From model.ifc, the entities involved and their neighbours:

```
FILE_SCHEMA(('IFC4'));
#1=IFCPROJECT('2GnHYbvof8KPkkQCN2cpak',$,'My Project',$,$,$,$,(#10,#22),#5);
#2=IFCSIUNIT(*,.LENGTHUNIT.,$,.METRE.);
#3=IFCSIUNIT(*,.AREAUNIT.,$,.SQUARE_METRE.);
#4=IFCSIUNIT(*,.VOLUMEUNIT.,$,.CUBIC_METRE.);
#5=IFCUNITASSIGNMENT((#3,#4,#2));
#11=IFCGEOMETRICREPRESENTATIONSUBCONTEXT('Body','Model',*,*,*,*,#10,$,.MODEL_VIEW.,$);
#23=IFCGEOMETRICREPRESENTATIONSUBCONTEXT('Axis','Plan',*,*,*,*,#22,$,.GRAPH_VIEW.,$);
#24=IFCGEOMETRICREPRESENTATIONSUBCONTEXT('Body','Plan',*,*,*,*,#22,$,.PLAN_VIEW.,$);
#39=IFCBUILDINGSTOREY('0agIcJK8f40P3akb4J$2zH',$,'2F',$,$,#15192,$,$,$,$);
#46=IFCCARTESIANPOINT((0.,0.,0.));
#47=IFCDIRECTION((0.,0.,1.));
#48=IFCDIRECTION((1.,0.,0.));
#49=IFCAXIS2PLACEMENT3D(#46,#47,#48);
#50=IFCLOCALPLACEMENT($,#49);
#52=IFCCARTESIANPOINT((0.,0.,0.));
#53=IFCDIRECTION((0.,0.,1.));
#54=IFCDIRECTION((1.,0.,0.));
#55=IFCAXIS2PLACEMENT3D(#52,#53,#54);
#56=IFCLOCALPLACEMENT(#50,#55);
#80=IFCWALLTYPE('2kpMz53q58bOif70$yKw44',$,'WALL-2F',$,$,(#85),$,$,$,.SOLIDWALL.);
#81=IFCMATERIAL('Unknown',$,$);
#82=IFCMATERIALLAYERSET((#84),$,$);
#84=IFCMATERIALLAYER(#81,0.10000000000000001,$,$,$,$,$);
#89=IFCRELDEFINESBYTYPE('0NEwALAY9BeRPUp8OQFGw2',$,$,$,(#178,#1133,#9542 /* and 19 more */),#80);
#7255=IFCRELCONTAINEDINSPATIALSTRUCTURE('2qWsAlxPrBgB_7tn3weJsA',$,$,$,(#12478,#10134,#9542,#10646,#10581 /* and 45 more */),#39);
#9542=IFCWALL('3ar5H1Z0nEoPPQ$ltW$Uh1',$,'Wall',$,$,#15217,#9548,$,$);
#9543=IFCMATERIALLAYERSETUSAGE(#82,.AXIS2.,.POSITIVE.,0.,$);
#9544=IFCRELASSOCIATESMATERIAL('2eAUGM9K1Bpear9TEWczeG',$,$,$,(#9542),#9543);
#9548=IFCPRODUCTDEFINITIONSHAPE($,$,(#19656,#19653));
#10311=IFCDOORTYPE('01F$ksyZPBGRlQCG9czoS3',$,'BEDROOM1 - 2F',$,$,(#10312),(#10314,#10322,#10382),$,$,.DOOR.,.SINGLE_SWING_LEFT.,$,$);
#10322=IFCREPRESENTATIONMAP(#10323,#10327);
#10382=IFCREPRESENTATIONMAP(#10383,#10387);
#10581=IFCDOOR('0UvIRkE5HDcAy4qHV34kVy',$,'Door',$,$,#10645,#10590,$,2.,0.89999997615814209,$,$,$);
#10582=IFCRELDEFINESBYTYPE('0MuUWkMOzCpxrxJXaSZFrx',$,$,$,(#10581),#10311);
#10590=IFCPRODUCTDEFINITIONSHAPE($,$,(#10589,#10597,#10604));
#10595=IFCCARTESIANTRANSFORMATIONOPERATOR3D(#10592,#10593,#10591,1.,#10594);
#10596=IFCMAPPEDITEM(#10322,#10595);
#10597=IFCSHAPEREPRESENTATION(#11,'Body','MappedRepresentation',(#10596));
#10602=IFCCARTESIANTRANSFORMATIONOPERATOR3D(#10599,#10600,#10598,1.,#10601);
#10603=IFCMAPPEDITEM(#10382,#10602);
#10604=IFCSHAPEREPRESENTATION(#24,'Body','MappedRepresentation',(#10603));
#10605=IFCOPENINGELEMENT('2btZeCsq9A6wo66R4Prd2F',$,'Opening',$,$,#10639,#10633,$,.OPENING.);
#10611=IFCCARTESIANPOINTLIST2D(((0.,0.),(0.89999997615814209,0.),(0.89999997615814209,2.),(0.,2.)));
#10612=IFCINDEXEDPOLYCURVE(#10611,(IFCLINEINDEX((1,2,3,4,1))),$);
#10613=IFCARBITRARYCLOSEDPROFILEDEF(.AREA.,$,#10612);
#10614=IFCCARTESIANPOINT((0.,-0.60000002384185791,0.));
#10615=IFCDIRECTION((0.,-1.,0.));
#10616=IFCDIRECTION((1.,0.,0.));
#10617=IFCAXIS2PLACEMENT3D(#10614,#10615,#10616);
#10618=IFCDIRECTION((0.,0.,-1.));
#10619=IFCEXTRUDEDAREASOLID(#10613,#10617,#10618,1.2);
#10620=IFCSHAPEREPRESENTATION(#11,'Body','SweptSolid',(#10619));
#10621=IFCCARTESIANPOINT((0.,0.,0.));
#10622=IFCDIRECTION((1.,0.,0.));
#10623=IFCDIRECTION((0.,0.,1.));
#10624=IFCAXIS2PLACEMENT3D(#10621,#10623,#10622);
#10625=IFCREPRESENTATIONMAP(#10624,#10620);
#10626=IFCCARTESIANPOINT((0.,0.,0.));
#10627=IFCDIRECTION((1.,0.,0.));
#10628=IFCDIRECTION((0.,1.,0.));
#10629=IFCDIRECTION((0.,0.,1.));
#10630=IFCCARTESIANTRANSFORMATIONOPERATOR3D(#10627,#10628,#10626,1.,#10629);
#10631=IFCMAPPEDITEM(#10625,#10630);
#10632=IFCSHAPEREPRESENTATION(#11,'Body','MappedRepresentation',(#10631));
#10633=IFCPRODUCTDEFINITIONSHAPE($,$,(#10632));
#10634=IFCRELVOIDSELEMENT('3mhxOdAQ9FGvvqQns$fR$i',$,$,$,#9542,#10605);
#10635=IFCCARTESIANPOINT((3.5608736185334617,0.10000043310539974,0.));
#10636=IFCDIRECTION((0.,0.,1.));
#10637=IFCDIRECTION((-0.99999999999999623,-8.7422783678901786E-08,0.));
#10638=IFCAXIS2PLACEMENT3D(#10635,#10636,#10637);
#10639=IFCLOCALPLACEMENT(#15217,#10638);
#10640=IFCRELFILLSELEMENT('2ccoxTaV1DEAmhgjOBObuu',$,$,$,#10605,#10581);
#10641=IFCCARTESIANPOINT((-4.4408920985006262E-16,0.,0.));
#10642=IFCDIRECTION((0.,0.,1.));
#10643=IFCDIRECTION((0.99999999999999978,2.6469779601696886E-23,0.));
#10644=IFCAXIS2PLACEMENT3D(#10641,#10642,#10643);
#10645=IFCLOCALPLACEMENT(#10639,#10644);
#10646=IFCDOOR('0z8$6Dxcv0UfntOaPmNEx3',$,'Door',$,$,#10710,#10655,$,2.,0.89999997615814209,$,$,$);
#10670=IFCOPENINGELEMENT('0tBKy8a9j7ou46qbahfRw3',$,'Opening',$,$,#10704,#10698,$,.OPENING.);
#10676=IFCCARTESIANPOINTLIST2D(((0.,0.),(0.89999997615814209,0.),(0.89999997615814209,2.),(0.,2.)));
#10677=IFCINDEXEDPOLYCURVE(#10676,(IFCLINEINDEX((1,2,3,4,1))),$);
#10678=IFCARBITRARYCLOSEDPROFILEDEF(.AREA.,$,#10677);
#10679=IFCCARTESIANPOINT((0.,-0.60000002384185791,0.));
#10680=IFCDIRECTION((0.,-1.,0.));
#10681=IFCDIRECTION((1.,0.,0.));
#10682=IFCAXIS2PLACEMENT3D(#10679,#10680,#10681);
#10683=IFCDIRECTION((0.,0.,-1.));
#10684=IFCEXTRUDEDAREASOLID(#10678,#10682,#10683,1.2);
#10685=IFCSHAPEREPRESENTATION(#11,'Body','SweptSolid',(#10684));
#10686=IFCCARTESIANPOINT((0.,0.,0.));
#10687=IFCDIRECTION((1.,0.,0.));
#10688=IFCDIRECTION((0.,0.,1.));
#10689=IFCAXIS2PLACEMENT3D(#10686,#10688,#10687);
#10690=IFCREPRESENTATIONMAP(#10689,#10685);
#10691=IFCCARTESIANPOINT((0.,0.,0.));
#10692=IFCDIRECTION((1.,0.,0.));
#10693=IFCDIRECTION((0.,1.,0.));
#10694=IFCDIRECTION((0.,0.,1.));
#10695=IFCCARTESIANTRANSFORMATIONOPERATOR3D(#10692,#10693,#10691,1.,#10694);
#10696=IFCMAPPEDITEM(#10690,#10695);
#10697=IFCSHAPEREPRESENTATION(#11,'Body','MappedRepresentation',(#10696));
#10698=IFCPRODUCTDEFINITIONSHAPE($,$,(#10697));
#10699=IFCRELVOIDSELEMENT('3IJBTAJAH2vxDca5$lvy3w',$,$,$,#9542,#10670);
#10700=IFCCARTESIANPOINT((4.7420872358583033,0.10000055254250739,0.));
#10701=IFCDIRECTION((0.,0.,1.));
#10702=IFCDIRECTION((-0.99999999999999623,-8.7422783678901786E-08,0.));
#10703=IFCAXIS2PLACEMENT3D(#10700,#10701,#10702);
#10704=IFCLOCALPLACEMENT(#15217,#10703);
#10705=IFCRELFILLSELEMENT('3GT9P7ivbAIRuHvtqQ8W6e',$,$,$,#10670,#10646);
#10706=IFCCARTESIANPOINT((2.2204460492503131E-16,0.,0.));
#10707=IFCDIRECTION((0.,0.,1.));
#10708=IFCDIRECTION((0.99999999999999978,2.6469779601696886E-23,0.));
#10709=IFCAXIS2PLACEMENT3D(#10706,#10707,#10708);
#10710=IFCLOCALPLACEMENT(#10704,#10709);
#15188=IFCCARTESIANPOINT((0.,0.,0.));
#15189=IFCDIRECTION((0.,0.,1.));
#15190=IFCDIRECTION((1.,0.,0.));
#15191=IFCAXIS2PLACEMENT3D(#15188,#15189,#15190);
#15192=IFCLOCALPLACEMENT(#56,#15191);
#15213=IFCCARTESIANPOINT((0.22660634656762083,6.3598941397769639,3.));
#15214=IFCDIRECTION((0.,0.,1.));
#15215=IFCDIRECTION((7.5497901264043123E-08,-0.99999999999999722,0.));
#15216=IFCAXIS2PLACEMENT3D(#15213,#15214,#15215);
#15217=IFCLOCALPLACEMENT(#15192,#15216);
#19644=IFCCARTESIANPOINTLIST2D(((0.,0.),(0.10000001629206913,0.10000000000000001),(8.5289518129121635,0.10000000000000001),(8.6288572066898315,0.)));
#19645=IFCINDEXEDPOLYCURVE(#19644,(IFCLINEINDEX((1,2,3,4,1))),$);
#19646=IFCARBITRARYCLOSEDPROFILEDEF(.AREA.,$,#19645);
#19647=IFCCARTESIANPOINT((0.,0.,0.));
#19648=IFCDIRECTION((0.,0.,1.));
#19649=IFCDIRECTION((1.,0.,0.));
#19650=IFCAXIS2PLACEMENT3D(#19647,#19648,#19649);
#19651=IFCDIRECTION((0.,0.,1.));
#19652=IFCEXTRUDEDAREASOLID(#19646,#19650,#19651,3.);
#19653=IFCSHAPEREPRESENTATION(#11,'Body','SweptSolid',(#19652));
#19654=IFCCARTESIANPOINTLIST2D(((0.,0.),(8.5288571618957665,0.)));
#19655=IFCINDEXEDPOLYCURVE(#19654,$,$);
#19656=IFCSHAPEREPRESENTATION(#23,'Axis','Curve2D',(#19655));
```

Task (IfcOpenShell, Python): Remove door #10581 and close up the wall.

```python
import ifcopenshell
import ifcopenshell.api.feature
import ifcopenshell.api.root
import ifcopenshell.geom
import ifcopenshell.util.shape

model = ifcopenshell.open("model.ifc")
settings = ifcopenshell.geom.settings()


def volume(element):
    """Net volume in cubic metres, openings subtracted."""
    shape = ifcopenshell.geom.create_shape(settings, element)
    return ifcopenshell.util.shape.get_volume(shape.geometry)


door = model.by_guid("0UvIRkE5HDcAy4qHV34kVy")
opening = door.FillsVoids[0].RelatingOpeningElement
wall = opening.VoidsElements[0].RelatingBuildingElement
before = volume(wall)

ifcopenshell.api.root.remove_product(model, product=door)
ifcopenshell.api.feature.remove_feature(model, feature=opening)

after = volume(wall)

print(f"wall volume {before:.3f} -> {after:.3f} m3")

model.write("model_v2.ifc")
```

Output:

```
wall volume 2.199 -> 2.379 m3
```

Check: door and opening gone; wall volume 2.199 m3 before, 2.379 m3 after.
